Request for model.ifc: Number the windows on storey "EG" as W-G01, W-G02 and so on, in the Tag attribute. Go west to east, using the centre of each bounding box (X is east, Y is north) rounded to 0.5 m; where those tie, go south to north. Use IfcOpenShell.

First a look at what the model holds.

```python
import ifcopenshell
import ifcopenshell.util.element
import ifcopenshell.util.placement

model = ifcopenshell.open("model.ifc")
print(model.schema)
storey = next(s for s in model.by_type("IfcBuildingStorey") if s.Name == "EG")
windows = [e for e in ifcopenshell.util.element.get_decomposition(storey) if e.is_a("IfcWindow")]
for e in sorted(windows, key=lambda e: e.id()):
    origin = ifcopenshell.util.placement.get_local_placement(e.ObjectPlacement)[:3, 3]
    print(e.id(), e.Tag, e.Name, origin.round(2) + 0.0, sep=" | ")
```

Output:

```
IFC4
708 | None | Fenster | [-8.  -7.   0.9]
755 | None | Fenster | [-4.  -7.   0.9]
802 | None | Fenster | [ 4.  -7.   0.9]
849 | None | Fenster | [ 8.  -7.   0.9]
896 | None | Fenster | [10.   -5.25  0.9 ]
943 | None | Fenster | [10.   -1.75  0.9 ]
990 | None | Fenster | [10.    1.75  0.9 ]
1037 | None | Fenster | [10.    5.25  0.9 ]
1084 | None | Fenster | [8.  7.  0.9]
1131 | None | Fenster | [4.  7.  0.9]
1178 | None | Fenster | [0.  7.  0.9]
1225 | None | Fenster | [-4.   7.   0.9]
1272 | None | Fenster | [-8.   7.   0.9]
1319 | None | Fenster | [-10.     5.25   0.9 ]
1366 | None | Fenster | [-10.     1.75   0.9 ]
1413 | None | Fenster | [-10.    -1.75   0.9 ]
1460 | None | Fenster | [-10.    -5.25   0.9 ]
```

```python
import ifcopenshell
import ifcopenshell.geom
import ifcopenshell.util.element
import ifcopenshell.util.shape

model = ifcopenshell.open("model.ifc")
settings = ifcopenshell.geom.settings()
settings.set("use-world-coords", True)


def centre(element):
    shape = ifcopenshell.geom.create_shape(settings, element)
    return ifcopenshell.util.shape.get_bbox_centroid(shape.geometry)


storey = next(s for s in model.by_type("IfcBuildingStorey") if s.Name == "EG")
windows = [e for e in ifcopenshell.util.element.get_decomposition(storey) if e.is_a("IfcWindow")]

# Insertion points can sit at a corner or the storey origin, so sort by the geometry (in metres).
centres = {e: centre(e) for e in windows}
windows.sort(key=lambda e: (round(centres[e][0] / 0.5), centres[e][1]))

for i, e in enumerate(windows, start=1):
    number = f"W-G{i:02d}"
    e.Tag = number
    print(e.id(), number)

model.write("model_updated.ifc")
```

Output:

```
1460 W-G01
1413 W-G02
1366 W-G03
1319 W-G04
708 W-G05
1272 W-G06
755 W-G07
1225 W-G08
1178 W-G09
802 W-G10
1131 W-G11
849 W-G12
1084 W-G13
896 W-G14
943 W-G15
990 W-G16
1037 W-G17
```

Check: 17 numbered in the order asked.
